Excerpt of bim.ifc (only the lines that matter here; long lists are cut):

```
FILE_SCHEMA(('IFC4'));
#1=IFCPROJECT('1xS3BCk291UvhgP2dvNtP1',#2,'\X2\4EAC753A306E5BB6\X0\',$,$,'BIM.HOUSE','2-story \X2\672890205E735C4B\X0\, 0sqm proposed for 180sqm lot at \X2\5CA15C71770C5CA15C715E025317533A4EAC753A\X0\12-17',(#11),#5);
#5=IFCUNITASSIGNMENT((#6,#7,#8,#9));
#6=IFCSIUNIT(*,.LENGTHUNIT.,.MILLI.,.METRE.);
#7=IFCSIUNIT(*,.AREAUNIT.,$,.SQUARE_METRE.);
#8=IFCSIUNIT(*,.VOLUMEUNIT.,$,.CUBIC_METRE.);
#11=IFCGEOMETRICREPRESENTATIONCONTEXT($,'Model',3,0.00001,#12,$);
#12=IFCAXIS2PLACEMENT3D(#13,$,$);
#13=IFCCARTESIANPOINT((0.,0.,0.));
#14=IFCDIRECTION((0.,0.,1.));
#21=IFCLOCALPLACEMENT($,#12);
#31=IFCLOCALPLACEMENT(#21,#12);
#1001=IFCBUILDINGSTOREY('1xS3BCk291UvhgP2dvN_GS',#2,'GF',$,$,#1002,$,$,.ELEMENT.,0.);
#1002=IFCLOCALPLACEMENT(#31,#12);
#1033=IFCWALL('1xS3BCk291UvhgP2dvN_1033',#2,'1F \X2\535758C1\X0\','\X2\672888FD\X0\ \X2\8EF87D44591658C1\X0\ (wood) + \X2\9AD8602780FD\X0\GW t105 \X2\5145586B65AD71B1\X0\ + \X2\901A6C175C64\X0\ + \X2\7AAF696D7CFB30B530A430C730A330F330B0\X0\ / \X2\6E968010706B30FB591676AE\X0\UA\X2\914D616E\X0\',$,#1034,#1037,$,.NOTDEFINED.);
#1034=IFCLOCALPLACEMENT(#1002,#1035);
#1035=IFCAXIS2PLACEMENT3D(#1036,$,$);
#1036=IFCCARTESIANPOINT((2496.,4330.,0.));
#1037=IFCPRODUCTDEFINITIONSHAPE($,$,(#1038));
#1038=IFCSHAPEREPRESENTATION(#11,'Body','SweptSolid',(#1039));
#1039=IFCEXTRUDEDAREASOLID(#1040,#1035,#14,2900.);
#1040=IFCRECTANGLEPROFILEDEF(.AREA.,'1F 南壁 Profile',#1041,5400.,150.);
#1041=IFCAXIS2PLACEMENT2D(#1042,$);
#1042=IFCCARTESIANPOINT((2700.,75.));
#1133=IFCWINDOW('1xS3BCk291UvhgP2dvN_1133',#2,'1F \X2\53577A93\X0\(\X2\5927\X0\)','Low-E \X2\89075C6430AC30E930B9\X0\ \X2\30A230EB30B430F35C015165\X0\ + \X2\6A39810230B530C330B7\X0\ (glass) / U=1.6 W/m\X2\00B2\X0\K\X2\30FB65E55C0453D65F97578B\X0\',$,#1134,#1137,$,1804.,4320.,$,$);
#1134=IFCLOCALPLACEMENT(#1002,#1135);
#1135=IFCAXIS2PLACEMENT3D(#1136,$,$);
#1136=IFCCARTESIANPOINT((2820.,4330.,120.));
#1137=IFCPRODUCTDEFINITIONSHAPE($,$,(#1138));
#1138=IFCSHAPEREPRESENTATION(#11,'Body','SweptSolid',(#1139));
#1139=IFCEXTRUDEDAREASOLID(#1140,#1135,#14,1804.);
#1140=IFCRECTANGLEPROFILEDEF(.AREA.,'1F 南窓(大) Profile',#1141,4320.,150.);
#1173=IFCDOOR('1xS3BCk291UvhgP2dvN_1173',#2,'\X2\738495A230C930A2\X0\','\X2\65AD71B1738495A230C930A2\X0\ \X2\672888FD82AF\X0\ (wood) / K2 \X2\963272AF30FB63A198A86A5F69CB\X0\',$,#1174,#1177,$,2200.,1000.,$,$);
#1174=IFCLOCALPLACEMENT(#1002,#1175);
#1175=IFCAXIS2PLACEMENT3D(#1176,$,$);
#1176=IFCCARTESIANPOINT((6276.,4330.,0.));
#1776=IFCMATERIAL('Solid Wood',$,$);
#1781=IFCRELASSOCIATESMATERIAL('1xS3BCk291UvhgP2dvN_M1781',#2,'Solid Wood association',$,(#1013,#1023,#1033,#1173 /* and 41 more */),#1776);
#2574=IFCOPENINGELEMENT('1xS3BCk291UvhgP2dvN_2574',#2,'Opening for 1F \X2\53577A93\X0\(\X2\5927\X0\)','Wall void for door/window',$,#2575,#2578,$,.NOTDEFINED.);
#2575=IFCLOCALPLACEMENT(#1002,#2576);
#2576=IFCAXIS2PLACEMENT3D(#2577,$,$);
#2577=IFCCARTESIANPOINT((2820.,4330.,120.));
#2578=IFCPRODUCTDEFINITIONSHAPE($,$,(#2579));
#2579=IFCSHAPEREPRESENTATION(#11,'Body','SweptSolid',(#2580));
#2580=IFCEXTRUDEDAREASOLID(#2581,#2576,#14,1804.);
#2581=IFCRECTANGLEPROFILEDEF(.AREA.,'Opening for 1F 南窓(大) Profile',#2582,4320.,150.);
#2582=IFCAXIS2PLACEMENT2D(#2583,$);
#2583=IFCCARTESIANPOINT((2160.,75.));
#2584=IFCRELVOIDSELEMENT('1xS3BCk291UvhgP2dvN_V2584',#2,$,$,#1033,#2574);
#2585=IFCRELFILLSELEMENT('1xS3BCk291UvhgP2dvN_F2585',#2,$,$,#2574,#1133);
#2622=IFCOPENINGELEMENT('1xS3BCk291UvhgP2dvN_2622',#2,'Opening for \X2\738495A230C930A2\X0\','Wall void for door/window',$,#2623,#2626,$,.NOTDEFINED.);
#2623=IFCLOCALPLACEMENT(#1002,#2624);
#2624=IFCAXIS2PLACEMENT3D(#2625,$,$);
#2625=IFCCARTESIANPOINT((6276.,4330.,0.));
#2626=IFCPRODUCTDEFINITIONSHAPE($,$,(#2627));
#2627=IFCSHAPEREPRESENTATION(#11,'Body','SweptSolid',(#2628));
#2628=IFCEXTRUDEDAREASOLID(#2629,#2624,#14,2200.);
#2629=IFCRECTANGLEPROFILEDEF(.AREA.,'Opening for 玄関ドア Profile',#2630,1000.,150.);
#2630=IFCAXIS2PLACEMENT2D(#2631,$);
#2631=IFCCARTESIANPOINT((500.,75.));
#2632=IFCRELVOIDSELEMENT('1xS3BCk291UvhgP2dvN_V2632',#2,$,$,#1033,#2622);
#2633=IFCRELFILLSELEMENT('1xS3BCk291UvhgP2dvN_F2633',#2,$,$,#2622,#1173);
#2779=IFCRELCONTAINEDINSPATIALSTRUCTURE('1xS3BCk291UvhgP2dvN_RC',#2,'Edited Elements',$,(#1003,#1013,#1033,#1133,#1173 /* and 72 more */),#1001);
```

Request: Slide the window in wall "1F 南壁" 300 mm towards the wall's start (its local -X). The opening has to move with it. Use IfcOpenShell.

```python
import ifcopenshell
import ifcopenshell.api.geometry
import ifcopenshell.util.placement
import ifcopenshell.util.unit

model = ifcopenshell.open("bim.ifc")
unit_scale = ifcopenshell.util.unit.calculate_unit_scale(model)

window = model.by_guid("1xS3BCk291UvhgP2dvN_1133")
opening = window.FillsVoids[0].RelatingOpeningElement
wall = opening.VoidsElements[0].RelatingBuildingElement

wall_matrix = ifcopenshell.util.placement.get_local_placement(wall.ObjectPlacement)
shift = wall_matrix[:3, 0] * -0.3 / unit_scale
before = ifcopenshell.util.placement.get_local_placement(window.ObjectPlacement)[:3, 3].copy()

# The window is not placed relative to its opening, so move both.
for product in (opening, window):
    matrix = ifcopenshell.util.placement.get_local_placement(product.ObjectPlacement)
    matrix[:3, 3] += shift
    ifcopenshell.api.geometry.edit_object_placement(model, product=product, matrix=matrix, is_si=False)

after = ifcopenshell.util.placement.get_local_placement(window.ObjectPlacement)[:3, 3]
print("window moved by", (after - before).round(3) + 0.0)

model.write("bim_v2.ifc")
```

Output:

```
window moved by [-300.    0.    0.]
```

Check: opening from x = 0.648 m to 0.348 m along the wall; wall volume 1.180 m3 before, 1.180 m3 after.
